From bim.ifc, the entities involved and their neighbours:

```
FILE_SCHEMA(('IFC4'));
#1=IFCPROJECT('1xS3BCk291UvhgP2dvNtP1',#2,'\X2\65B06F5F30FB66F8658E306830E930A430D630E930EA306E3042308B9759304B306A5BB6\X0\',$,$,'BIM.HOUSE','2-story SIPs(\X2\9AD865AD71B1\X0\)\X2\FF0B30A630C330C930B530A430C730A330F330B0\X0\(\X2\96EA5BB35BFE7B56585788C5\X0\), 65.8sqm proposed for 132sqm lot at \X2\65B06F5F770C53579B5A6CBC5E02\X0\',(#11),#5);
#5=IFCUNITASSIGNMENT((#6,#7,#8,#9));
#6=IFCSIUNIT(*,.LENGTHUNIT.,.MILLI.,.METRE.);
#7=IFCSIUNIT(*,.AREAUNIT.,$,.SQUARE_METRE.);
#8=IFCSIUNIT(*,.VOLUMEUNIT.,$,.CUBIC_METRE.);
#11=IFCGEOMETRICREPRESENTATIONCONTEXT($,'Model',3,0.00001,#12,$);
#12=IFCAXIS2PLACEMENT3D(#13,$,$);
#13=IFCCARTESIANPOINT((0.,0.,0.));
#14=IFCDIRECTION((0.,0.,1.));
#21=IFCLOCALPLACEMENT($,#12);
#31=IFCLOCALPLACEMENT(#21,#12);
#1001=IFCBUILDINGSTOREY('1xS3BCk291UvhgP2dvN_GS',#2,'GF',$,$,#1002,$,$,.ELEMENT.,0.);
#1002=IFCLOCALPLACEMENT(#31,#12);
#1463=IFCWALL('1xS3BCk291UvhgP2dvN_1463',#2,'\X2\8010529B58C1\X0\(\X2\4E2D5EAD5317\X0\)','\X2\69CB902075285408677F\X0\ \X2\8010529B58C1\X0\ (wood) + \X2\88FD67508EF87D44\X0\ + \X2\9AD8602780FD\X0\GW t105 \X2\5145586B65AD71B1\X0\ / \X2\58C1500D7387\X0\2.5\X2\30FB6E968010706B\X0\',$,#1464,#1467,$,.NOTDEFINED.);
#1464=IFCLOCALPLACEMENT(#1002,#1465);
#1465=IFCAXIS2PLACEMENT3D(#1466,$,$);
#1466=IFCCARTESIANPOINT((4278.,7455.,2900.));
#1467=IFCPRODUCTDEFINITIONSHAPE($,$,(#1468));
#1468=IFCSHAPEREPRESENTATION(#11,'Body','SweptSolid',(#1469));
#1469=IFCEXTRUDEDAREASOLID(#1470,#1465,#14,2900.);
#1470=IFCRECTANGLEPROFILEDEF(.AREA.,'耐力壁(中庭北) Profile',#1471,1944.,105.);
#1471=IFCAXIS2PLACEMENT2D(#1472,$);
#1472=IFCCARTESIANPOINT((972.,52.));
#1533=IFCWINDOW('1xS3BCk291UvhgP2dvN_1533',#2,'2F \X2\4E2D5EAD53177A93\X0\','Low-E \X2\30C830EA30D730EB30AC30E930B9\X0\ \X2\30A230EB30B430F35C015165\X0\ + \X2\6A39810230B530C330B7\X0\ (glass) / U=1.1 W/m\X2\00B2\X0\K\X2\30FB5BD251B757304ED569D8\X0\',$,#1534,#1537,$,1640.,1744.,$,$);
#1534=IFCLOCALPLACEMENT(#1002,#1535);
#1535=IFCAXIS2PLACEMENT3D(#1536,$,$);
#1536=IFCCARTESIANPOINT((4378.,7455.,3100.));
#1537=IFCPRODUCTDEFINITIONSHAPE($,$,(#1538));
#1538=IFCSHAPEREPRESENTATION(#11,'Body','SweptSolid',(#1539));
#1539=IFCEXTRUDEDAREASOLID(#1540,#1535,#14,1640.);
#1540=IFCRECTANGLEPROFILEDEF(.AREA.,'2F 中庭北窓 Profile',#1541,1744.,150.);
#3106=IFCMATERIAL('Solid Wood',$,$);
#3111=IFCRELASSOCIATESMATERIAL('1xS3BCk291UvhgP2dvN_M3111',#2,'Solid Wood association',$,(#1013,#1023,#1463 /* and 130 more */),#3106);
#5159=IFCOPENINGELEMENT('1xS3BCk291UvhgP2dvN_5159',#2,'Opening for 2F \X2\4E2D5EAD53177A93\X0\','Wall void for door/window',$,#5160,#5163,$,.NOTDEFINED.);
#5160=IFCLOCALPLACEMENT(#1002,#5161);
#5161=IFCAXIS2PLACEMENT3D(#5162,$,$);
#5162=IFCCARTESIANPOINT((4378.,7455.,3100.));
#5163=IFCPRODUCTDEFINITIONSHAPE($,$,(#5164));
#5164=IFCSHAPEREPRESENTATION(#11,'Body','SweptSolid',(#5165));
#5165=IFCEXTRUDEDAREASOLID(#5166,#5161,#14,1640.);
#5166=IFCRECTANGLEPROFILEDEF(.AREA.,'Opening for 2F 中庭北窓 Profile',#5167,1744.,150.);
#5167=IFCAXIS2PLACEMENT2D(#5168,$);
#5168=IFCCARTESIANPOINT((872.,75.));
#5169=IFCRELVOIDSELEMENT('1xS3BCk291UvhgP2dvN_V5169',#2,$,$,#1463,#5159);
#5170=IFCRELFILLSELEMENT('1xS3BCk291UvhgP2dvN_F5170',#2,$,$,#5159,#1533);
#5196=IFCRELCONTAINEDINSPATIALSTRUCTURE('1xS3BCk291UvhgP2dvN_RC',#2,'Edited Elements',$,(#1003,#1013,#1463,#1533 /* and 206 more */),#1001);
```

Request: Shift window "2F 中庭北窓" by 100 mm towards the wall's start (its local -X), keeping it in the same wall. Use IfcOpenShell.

```python
import ifcopenshell
import ifcopenshell.api.geometry
import ifcopenshell.util.placement
import ifcopenshell.util.unit

model = ifcopenshell.open("bim.ifc")
unit_scale = ifcopenshell.util.unit.calculate_unit_scale(model)

window = model.by_guid("1xS3BCk291UvhgP2dvN_1533")
opening = window.FillsVoids[0].RelatingOpeningElement
wall = opening.VoidsElements[0].RelatingBuildingElement

wall_matrix = ifcopenshell.util.placement.get_local_placement(wall.ObjectPlacement)
shift = wall_matrix[:3, 0] * -0.1 / unit_scale
before = ifcopenshell.util.placement.get_local_placement(window.ObjectPlacement)[:3, 3].copy()

# The window is not placed relative to its opening, so move both.
for product in (opening, window):
    matrix = ifcopenshell.util.placement.get_local_placement(product.ObjectPlacement)
    matrix[:3, 3] += shift
    ifcopenshell.api.geometry.edit_object_placement(model, product=product, matrix=matrix, is_si=False)

after = ifcopenshell.util.placement.get_local_placement(window.ObjectPlacement)[:3, 3]
print("window moved by", (after - before).round(3) + 0.0)

model.write("bim_v2.ifc")
```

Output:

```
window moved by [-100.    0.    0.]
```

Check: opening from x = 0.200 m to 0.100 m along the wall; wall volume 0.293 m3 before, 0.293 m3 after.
